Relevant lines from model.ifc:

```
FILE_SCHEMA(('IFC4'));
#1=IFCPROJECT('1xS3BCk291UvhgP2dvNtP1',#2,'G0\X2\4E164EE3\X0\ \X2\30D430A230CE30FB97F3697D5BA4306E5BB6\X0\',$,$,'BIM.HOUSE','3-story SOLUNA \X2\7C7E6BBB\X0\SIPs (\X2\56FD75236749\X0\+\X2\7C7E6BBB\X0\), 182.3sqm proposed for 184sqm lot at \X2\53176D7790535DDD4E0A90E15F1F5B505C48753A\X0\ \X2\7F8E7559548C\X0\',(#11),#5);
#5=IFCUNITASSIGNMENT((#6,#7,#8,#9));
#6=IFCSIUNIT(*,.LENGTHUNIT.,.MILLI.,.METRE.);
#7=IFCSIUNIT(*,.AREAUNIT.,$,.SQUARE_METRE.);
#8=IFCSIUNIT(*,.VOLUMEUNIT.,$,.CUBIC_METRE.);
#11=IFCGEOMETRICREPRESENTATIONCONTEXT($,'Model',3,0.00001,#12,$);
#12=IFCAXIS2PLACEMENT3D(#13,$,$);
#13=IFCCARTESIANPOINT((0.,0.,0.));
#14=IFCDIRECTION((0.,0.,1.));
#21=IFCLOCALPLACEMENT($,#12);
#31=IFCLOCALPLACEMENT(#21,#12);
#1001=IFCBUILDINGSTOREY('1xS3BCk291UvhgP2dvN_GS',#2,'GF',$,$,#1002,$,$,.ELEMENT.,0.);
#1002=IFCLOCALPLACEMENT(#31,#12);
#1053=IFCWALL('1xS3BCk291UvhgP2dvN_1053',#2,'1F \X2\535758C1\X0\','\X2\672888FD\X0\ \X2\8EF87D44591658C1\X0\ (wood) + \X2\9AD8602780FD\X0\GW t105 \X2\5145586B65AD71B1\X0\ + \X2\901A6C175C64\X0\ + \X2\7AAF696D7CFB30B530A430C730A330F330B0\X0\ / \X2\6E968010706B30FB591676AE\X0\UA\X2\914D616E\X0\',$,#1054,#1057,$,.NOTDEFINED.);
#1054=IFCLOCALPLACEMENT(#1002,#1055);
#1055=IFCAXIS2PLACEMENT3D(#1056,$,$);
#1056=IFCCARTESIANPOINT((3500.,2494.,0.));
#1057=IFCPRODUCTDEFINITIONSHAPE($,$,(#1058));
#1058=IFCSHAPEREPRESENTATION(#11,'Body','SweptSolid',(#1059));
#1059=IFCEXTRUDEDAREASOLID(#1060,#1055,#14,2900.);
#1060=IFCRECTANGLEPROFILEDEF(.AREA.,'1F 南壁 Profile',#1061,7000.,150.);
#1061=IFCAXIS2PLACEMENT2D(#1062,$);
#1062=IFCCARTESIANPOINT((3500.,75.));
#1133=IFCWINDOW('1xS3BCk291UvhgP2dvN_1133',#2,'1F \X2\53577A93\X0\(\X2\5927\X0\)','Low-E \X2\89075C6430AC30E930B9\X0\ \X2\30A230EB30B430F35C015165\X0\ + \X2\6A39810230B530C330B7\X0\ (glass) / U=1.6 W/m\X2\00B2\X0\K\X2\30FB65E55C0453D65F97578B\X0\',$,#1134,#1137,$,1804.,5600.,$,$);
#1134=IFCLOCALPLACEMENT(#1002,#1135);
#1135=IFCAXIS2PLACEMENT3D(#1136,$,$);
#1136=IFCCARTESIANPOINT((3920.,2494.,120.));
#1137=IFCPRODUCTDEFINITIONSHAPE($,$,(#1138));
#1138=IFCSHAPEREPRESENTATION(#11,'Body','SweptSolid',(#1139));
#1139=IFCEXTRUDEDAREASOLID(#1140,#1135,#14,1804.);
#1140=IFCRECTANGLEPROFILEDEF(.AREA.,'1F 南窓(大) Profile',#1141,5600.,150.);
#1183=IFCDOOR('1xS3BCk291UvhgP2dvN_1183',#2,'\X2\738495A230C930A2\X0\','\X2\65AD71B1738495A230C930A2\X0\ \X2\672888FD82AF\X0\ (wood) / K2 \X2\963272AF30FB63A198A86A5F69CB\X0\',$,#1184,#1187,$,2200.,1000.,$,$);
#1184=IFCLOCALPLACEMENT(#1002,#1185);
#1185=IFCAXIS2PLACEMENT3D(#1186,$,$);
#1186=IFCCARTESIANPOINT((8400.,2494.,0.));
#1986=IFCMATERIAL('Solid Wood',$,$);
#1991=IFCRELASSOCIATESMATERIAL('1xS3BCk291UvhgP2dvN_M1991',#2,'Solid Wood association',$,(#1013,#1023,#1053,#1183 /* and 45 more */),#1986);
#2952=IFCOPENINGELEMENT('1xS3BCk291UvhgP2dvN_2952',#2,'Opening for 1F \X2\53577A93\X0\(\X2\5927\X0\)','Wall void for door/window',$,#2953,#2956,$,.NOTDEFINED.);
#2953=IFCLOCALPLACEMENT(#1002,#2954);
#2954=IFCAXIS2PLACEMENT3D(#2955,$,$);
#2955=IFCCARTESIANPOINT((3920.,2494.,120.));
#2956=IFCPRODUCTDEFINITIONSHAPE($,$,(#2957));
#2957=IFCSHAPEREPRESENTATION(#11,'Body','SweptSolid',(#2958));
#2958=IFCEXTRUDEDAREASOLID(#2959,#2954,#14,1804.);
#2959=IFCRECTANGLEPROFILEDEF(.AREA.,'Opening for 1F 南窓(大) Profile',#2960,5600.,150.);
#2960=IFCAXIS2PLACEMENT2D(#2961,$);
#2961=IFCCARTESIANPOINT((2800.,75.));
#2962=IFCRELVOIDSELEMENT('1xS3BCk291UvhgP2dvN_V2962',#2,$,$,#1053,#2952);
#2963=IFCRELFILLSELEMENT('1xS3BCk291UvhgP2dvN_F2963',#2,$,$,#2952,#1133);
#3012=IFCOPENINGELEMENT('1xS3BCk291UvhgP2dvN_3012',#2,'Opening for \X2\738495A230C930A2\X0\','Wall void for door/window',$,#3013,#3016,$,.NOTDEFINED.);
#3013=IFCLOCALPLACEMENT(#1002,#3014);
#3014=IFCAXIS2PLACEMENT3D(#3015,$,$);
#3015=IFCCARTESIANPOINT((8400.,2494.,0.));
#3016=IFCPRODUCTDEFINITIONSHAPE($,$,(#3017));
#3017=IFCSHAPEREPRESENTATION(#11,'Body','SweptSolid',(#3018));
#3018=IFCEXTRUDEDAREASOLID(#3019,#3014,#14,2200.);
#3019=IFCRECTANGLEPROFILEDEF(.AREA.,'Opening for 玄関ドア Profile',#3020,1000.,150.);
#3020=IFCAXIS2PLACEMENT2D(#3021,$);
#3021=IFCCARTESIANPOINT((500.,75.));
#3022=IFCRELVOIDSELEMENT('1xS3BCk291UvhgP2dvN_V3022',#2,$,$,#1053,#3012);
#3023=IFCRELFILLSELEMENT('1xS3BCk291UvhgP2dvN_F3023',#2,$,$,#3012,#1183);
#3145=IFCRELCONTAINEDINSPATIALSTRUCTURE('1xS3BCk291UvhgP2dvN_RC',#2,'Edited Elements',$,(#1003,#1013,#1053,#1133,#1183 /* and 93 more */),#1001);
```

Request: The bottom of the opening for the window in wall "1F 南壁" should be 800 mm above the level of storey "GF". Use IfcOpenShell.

```python
import numpy as np
import ifcopenshell
import ifcopenshell.api.geometry
import ifcopenshell.geom
import ifcopenshell.util.element
import ifcopenshell.util.placement
import ifcopenshell.util.shape
import ifcopenshell.util.unit

model = ifcopenshell.open("model.ifc")
unit_scale = ifcopenshell.util.unit.calculate_unit_scale(model)

window = model.by_guid("1xS3BCk291UvhgP2dvN_1133")
opening = window.FillsVoids[0].RelatingOpeningElement
storey = ifcopenshell.util.element.get_container(window, ifc_class="IfcBuildingStorey")
level = ifcopenshell.util.placement.get_local_placement(storey.ObjectPlacement)[2, 3]

# The opening's origin need not be at the sill, so measure its lowest point.
shape = ifcopenshell.geom.create_shape(ifcopenshell.geom.settings(), opening)
bottom = ifcopenshell.util.shape.get_shape_bottom_elevation(shape, shape.geometry) / unit_scale
dz = level + 0.8 / unit_scale - bottom

shift = np.array([0.0, 0.0, dz])
# The window is not placed relative to its opening, so move both.
for product in (opening, window):
    matrix = ifcopenshell.util.placement.get_local_placement(product.ObjectPlacement)
    matrix[:3, 3] += shift
    ifcopenshell.api.geometry.edit_object_placement(model, product=product, matrix=matrix, is_si=False)

print(f"moved by {dz * unit_scale:+.3f} m")

model.write("model_rev.ifc")
```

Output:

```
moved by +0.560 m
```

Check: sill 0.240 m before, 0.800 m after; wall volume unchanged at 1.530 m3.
